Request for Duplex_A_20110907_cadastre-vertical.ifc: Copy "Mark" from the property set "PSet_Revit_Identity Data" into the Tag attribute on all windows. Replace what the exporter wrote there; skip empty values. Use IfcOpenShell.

First a look at what the model holds.

```python
import ifcopenshell
import ifcopenshell.util.element

model = ifcopenshell.open("Duplex_A_20110907_cadastre-vertical.ifc")
print(model.schema)
windows = model.by_type("IfcWindow")
print(len(windows), "windows")
for e in windows[:8]:
    source = ifcopenshell.util.element.get_pset(e, "PSet_Revit_Identity Data", "Mark")
    target = e.Tag
    print(e.id(), repr(source), repr(target), sep=" | ")
```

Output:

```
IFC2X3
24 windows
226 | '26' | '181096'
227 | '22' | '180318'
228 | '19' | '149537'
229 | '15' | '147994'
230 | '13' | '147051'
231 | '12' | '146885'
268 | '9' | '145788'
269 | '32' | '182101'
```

```python
import ifcopenshell
import ifcopenshell.util.element

model = ifcopenshell.open("Duplex_A_20110907_cadastre-vertical.ifc")

count = 0
for e in model.by_type("IfcWindow"):
    value = ifcopenshell.util.element.get_pset(e, "PSet_Revit_Identity Data", "Mark")
    current = e.Tag
    if not value or not value.strip() or current == value:
        continue
    e.Tag = value
    count += 1

print(count, "windows updated")

model.write("Duplex_A_20110907_cadastre-vertical_v2.ifc")
```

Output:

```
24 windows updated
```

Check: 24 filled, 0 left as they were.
